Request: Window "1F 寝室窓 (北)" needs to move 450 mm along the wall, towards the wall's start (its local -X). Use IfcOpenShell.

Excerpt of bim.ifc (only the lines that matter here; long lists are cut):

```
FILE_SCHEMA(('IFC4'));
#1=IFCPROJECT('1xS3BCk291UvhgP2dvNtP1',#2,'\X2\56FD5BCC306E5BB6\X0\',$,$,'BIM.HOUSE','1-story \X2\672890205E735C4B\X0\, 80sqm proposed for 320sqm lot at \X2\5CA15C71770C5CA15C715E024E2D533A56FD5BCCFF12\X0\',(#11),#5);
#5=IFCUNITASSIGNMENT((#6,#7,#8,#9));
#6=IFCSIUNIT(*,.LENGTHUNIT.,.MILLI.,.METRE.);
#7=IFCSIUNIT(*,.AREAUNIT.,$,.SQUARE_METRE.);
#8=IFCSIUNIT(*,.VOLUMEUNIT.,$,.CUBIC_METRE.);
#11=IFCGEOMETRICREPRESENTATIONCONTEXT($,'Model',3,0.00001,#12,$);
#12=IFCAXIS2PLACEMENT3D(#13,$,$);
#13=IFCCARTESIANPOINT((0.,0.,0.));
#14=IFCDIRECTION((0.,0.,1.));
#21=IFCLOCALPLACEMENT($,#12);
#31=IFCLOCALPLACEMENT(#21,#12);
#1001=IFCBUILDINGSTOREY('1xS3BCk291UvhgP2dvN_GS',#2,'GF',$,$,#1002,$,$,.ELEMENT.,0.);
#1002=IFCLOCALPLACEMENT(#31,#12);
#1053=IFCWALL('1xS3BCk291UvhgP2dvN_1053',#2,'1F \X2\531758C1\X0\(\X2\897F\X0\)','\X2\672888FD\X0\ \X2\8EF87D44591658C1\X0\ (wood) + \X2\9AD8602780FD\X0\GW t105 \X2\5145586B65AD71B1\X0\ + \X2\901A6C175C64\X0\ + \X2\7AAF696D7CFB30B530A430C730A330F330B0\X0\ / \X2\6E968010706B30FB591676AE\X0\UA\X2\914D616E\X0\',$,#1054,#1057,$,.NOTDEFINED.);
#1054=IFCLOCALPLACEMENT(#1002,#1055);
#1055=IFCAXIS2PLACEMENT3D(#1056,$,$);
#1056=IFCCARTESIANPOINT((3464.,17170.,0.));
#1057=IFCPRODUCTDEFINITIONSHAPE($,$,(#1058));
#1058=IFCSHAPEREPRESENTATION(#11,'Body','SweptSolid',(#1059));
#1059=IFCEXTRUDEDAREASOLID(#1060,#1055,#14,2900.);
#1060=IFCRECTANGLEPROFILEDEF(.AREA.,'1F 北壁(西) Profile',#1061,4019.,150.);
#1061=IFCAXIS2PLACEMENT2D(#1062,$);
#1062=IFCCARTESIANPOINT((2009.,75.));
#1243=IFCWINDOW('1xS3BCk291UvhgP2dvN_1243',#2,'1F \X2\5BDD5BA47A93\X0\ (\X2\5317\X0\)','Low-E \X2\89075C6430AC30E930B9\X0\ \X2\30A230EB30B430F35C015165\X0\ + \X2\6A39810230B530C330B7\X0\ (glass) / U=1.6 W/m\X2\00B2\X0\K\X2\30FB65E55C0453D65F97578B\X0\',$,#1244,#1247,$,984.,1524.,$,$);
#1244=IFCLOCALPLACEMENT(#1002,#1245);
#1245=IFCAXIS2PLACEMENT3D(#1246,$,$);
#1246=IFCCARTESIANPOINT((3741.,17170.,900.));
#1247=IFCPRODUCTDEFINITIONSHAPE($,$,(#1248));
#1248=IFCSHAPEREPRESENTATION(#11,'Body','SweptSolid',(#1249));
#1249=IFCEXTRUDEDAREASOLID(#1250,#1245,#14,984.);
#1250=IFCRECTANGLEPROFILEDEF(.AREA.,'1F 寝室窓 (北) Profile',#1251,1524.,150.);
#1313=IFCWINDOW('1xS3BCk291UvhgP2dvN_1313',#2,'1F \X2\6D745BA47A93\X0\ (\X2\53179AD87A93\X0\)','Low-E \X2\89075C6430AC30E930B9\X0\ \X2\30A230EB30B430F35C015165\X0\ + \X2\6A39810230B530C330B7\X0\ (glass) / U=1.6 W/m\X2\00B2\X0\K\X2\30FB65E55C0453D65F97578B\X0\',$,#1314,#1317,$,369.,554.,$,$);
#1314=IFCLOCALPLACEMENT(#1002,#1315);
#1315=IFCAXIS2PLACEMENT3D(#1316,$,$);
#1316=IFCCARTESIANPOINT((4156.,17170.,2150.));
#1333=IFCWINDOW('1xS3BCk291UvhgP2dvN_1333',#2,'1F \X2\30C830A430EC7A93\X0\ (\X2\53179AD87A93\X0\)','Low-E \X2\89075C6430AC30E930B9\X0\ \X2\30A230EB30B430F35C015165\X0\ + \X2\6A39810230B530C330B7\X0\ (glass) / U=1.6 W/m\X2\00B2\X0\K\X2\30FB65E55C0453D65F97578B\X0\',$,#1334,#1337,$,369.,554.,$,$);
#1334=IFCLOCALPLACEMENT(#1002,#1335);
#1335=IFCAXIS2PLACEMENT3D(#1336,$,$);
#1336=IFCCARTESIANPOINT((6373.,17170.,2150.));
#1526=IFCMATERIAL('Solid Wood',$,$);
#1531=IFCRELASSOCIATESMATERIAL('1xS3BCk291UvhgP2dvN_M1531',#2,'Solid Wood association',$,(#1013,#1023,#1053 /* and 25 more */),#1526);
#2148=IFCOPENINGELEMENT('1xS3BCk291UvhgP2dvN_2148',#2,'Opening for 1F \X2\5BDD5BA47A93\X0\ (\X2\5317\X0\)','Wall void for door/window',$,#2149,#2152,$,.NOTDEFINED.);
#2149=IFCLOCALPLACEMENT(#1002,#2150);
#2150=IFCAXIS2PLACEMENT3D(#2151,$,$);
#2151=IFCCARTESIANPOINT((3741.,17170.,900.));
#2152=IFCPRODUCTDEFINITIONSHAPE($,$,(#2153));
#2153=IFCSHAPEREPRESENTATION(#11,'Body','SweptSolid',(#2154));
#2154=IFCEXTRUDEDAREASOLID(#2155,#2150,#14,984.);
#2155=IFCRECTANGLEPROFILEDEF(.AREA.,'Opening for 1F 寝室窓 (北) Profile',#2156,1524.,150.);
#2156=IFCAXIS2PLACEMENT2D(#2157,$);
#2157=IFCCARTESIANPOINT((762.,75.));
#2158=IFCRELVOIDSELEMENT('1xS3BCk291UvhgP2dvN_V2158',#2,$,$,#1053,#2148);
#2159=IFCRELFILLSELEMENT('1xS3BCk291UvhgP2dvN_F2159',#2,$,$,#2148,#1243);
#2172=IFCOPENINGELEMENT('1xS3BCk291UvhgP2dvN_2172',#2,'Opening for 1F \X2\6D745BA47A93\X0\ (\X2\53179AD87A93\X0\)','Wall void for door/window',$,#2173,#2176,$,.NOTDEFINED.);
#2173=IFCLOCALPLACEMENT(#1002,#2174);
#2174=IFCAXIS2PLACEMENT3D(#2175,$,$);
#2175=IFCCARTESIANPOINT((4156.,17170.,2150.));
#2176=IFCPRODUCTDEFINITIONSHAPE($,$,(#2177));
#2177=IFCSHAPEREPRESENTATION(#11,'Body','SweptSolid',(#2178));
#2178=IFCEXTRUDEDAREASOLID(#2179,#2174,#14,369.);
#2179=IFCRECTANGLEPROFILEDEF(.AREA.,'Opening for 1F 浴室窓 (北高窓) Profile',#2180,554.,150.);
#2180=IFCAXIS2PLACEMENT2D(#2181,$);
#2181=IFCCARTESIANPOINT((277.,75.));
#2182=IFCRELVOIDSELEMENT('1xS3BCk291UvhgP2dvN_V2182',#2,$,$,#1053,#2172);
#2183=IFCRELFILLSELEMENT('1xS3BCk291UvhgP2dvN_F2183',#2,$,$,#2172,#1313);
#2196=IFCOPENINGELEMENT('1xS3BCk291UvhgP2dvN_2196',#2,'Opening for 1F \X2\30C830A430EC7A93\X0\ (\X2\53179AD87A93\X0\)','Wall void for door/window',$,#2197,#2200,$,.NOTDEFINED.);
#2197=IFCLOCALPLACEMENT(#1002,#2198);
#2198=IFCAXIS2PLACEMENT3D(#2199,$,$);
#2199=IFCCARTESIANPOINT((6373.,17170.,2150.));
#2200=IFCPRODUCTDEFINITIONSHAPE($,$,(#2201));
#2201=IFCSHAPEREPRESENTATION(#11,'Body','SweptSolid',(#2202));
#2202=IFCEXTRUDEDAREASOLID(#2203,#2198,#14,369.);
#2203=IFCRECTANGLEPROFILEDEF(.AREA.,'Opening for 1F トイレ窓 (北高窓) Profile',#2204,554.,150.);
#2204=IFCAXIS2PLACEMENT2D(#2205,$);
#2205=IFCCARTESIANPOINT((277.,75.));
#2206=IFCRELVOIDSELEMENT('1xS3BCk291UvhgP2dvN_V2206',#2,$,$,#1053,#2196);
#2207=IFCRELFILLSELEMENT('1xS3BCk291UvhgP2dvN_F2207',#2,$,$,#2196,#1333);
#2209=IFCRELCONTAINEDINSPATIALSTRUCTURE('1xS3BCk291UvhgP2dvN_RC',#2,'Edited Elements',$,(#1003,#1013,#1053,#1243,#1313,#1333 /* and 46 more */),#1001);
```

```python
import ifcopenshell
import ifcopenshell.api.geometry
import ifcopenshell.util.placement

model = ifcopenshell.open("bim.ifc")

window = model.by_id(1243)
opening = window.FillsVoids[0].RelatingOpeningElement
wall = opening.VoidsElements[0].RelatingBuildingElement

wall_matrix = ifcopenshell.util.placement.get_local_placement(wall.ObjectPlacement)
shift = wall_matrix[:3, 0] * -450.0
before = ifcopenshell.util.placement.get_local_placement(window.ObjectPlacement)[:3, 3].copy()

# The window is not placed relative to its opening, so move both.
for product in (opening, window):
    matrix = ifcopenshell.util.placement.get_local_placement(product.ObjectPlacement)
    matrix[:3, 3] += shift
    ifcopenshell.api.geometry.edit_object_placement(model, product=product, matrix=matrix, is_si=False)

after = ifcopenshell.util.placement.get_local_placement(window.ObjectPlacement)[:3, 3]
print("window moved by", (after - before).round(3) + 0.0)

model.write("bim-out.ifc")
```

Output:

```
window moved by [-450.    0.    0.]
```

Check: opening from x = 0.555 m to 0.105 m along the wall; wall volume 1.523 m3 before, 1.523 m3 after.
